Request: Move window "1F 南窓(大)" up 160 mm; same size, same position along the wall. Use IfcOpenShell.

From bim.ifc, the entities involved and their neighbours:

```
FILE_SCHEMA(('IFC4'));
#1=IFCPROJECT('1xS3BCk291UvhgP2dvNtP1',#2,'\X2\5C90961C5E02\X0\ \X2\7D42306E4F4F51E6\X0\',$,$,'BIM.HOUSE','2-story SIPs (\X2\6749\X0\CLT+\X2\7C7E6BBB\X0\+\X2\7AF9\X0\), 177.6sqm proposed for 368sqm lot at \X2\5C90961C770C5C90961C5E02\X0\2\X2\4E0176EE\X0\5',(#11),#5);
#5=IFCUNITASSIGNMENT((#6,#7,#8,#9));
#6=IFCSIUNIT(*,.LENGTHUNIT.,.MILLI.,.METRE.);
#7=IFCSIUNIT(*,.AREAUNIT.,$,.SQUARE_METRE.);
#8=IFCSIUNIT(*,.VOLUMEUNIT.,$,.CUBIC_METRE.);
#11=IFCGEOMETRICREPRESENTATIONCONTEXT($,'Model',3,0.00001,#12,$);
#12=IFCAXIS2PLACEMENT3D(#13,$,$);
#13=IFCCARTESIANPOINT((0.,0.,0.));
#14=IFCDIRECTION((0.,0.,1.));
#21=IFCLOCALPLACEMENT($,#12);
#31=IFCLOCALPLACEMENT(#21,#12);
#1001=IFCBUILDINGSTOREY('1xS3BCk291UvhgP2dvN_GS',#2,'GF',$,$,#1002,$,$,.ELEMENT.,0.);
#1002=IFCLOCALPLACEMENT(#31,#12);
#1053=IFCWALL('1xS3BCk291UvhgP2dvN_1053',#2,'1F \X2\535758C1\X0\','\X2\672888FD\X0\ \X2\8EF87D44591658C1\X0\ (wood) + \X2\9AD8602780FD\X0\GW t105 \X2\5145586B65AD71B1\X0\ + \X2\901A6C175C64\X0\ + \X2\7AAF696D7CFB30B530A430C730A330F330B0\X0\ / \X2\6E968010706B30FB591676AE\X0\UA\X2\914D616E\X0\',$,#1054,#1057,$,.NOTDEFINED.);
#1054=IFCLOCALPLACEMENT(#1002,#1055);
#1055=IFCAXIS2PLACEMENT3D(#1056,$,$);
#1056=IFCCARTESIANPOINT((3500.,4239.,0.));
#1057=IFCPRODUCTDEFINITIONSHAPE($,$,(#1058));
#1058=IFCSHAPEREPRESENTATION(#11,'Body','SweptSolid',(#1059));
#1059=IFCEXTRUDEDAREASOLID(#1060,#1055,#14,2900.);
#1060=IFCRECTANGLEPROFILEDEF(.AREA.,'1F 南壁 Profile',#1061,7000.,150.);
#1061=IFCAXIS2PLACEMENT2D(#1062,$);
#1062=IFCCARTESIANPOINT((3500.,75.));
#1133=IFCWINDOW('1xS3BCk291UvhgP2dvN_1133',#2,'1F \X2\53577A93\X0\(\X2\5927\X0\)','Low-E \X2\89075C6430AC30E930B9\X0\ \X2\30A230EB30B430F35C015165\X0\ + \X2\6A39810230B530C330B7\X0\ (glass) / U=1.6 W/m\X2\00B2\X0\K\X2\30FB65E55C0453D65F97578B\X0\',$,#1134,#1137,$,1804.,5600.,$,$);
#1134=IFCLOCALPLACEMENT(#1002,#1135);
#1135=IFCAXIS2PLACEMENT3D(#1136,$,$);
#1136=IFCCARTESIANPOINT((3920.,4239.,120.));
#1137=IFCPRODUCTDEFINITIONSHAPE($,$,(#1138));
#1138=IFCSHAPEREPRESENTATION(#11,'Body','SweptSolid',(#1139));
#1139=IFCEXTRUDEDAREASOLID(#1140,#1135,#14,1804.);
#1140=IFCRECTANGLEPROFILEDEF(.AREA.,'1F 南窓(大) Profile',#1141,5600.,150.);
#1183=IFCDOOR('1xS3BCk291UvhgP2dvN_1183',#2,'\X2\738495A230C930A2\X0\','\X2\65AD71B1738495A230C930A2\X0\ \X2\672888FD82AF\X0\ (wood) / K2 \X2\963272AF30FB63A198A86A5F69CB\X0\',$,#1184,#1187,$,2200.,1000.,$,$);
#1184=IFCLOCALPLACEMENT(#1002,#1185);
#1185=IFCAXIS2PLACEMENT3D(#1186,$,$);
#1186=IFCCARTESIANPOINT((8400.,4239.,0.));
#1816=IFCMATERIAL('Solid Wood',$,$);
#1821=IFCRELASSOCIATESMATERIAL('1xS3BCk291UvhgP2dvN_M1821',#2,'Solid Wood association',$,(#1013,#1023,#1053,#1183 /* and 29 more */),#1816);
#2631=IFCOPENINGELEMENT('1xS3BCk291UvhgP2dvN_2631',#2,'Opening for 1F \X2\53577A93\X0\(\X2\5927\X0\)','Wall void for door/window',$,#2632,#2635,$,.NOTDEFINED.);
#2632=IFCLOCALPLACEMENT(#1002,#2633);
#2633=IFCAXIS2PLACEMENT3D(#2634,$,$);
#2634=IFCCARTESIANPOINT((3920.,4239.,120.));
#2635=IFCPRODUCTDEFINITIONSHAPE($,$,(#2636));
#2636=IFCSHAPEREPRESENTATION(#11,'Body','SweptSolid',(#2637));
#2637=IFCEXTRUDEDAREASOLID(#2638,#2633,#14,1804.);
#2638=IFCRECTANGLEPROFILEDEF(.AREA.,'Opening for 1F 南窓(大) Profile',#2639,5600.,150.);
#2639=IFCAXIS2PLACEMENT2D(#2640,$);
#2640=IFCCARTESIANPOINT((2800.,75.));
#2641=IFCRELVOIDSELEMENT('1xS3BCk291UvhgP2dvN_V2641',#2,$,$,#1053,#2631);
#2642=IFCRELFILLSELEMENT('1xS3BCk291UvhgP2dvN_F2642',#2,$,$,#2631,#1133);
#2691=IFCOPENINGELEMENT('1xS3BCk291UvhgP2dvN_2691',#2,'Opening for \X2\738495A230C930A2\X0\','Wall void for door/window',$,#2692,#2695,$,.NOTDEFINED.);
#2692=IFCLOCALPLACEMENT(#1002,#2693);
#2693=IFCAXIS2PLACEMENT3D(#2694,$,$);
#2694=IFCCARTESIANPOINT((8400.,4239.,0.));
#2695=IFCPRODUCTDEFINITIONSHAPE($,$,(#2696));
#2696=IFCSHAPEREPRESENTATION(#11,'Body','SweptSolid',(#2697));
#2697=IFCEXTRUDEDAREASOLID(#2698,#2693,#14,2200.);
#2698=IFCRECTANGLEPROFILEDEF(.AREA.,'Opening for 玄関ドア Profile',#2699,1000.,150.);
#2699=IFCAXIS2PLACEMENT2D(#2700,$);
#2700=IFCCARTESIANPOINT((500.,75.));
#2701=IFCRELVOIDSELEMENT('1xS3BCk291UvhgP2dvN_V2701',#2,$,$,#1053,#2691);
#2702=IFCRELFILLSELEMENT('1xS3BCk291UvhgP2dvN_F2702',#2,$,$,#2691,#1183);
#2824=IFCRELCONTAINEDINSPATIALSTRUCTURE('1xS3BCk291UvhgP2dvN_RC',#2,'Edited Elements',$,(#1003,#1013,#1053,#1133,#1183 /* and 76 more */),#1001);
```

```python
import numpy as np
import ifcopenshell
import ifcopenshell.api.geometry
import ifcopenshell.util.placement
import ifcopenshell.util.unit

model = ifcopenshell.open("bim.ifc")
unit_scale = ifcopenshell.util.unit.calculate_unit_scale(model)

window = model.by_guid("1xS3BCk291UvhgP2dvN_1133")
opening = window.FillsVoids[0].RelatingOpeningElement
dz = 0.16 / unit_scale

shift = np.array([0.0, 0.0, dz])
# The window is not placed relative to its opening, so move both.
for product in (opening, window):
    matrix = ifcopenshell.util.placement.get_local_placement(product.ObjectPlacement)
    matrix[:3, 3] += shift
    ifcopenshell.api.geometry.edit_object_placement(model, product=product, matrix=matrix, is_si=False)

print(f"moved by {dz * unit_scale:+.3f} m")

model.write("bim_rev.ifc")
```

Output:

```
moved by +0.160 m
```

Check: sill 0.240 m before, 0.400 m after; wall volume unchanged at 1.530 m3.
